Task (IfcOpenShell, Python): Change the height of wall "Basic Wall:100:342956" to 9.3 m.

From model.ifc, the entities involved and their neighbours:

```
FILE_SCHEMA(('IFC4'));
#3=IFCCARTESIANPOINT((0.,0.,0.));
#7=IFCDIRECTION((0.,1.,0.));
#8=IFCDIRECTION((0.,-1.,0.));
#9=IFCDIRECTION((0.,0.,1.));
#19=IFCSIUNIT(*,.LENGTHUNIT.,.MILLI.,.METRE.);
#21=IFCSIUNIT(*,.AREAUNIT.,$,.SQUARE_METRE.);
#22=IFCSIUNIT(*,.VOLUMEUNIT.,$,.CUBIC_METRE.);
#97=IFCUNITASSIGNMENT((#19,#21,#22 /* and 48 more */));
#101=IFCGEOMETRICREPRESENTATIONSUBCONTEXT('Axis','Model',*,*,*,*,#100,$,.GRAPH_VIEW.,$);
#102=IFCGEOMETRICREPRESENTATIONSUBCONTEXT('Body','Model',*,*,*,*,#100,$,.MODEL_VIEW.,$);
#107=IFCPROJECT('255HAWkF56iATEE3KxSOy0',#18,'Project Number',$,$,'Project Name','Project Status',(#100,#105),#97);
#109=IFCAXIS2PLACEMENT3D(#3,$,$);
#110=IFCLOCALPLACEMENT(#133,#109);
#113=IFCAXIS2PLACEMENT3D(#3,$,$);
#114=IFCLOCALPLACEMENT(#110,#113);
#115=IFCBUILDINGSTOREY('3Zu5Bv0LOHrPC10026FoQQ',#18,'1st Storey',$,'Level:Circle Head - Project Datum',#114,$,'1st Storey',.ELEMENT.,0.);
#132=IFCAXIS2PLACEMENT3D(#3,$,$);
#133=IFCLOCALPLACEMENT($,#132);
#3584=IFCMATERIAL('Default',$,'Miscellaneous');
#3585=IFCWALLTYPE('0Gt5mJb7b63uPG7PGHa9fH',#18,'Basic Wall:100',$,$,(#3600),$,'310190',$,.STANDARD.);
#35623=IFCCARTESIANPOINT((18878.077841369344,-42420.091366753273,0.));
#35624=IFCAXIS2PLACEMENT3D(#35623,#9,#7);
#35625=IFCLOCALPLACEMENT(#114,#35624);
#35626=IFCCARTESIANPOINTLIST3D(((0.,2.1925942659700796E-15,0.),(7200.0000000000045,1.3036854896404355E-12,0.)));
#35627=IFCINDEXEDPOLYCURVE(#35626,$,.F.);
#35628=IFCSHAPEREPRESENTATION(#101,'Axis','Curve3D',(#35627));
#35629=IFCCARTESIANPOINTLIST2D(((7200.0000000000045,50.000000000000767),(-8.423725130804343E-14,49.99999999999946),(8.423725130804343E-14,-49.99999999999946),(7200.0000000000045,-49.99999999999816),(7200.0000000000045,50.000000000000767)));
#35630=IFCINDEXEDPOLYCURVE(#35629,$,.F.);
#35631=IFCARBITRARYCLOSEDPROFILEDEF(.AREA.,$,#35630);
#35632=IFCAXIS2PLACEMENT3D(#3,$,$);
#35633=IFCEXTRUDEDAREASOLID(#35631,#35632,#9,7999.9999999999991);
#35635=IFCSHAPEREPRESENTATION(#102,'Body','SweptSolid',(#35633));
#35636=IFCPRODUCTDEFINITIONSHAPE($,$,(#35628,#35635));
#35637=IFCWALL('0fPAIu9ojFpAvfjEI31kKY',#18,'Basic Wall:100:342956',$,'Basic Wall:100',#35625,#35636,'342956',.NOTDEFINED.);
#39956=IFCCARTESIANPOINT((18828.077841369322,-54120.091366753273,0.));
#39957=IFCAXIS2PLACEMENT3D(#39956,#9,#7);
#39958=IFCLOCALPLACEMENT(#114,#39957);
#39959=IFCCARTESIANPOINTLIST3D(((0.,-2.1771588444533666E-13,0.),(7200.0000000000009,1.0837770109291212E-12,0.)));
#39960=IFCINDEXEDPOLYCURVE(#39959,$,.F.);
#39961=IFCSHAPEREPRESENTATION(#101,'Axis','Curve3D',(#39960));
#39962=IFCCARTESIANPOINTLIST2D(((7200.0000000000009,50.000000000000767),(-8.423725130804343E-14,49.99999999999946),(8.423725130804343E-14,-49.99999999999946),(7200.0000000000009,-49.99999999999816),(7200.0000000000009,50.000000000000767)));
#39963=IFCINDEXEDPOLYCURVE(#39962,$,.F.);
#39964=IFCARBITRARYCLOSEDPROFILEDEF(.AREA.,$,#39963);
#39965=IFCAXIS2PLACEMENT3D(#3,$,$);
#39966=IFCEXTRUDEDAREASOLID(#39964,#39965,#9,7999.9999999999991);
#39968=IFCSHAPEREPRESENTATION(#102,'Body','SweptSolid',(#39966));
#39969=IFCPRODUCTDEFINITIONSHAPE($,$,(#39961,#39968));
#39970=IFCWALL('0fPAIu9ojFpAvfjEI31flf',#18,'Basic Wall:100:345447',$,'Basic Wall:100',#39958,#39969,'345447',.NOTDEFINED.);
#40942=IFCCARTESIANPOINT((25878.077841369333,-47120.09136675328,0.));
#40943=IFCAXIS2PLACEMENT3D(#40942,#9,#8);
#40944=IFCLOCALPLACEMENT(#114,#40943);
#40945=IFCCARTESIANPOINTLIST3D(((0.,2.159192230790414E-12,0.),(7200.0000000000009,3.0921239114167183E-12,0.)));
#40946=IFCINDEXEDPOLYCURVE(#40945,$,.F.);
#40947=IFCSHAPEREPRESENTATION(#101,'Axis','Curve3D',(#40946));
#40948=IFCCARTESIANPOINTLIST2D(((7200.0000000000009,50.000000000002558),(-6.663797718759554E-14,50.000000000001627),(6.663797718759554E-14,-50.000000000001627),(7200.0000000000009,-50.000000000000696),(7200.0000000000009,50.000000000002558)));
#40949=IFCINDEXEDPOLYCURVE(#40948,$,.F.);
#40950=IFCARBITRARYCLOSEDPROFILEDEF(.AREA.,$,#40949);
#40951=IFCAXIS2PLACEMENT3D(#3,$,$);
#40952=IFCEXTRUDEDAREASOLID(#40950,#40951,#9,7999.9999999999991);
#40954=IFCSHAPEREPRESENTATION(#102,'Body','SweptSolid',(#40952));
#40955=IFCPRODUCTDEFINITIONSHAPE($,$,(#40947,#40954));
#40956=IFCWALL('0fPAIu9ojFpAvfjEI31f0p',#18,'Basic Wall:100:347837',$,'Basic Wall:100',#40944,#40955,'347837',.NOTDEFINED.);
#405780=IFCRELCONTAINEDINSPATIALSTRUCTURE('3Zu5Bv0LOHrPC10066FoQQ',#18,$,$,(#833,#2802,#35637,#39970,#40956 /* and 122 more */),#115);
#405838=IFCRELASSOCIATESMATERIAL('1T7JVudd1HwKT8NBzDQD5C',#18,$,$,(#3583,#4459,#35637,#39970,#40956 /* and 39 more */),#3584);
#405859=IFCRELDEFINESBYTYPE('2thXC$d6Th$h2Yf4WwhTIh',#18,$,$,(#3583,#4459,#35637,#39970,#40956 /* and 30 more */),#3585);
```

```python
import ifcopenshell
import ifcopenshell.geom
import ifcopenshell.util.representation
import ifcopenshell.util.shape

model = ifcopenshell.open("model.ifc")
settings = ifcopenshell.geom.settings()


def volume(element):
    """Net volume in cubic metres, openings subtracted."""
    shape = ifcopenshell.geom.create_shape(settings, element)
    return ifcopenshell.util.shape.get_volume(shape.geometry)


wall = model.by_id(35637)
before = volume(wall)

body = ifcopenshell.util.representation.get_representation(wall, "Model", "Body")
solid = body.Items[0]
old_height = solid.Depth
solid.Depth = 9300.0
after = volume(wall)

print(f"height {old_height:g} -> {solid.Depth:g}, volume {before:.3f} -> {after:.3f} m3")

model.write("model-out.ifc")
```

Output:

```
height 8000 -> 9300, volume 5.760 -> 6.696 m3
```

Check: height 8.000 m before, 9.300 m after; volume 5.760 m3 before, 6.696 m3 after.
